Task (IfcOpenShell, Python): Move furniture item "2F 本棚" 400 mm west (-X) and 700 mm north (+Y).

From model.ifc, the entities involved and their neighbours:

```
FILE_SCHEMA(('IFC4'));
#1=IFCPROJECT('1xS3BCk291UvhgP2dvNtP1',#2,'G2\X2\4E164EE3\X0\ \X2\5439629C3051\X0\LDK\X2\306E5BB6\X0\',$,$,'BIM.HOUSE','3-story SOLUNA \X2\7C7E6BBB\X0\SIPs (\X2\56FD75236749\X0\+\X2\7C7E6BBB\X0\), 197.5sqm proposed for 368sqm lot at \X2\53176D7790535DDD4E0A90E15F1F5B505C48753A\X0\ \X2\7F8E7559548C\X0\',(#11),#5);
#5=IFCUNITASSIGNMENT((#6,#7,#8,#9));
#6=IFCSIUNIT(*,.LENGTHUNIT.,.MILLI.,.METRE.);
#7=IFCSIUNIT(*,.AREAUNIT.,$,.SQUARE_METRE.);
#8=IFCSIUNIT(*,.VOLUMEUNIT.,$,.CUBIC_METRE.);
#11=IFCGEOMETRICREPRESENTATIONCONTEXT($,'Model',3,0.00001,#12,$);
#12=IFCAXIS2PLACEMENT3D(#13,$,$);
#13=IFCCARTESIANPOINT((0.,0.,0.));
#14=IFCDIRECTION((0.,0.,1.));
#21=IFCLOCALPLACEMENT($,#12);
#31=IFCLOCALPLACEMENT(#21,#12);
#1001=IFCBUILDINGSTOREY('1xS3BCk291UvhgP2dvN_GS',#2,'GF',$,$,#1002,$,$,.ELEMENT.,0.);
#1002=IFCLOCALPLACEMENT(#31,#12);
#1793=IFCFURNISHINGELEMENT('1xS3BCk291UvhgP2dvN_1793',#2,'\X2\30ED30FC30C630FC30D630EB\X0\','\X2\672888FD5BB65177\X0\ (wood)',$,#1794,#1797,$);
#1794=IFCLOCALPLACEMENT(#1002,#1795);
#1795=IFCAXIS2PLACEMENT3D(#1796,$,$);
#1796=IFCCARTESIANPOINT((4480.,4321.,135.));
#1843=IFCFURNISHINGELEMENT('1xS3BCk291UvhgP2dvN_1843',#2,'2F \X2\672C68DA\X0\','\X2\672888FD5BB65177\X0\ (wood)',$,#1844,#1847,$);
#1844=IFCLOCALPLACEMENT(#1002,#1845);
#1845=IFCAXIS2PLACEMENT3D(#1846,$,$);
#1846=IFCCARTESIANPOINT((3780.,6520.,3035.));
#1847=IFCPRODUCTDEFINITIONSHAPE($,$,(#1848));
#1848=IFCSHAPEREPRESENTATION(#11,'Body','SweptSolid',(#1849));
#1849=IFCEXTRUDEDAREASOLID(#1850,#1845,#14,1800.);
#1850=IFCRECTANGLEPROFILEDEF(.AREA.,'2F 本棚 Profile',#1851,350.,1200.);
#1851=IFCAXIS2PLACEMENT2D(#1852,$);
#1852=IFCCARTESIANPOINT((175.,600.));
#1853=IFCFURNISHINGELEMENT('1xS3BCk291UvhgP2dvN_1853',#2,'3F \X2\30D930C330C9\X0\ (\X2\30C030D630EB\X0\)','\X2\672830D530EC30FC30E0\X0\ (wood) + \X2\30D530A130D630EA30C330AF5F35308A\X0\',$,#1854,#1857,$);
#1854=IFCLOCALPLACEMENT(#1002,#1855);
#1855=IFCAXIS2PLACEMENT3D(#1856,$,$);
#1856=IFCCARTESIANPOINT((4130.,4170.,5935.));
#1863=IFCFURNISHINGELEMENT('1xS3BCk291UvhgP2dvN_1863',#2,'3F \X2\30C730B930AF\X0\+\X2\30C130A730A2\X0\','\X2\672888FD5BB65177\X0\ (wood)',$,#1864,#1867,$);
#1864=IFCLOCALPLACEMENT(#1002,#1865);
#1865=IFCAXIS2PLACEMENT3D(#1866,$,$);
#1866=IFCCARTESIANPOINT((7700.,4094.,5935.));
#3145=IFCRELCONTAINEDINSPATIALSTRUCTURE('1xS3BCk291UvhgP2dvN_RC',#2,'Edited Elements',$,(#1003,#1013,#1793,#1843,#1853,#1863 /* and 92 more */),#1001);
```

```python
import ifcopenshell
import ifcopenshell.api.geometry
import ifcopenshell.util.placement
import ifcopenshell.util.unit

model = ifcopenshell.open("model.ifc")
unit_scale = ifcopenshell.util.unit.calculate_unit_scale(model)

item = model.by_id(1843)
matrix = ifcopenshell.util.placement.get_local_placement(item.ObjectPlacement)
matrix[0, 3] -= 0.4 / unit_scale
matrix[1, 3] += 0.7 / unit_scale
ifcopenshell.api.geometry.edit_object_placement(model, product=item, matrix=matrix, is_si=False)

print(ifcopenshell.util.placement.get_local_placement(item.ObjectPlacement).round(3) + 0.0)

model.write("model_updated.ifc")
```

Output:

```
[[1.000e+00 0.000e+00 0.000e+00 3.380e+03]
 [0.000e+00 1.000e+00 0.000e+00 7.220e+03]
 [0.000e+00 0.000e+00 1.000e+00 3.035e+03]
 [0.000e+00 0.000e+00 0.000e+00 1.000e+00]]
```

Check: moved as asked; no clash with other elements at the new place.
